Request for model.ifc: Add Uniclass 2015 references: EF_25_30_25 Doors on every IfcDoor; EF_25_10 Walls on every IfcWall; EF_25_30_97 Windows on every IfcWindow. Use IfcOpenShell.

First a look at what the model holds.

```python
import ifcopenshell

model = ifcopenshell.open("model.ifc")
print(model.schema)
print("classifications:", [c.Name for c in model.by_type("IfcClassification")])
for ifc_class in ("IfcDoor", "IfcRoof", "IfcStair", "IfcWall", "IfcWindow"):
    print(ifc_class, len(model.by_type(ifc_class)))
```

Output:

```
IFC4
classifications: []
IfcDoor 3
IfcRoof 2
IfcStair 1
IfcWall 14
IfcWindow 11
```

```python
import ifcopenshell
import ifcopenshell.api.classification

model = ifcopenshell.open("model.ifc")

system = ifcopenshell.api.classification.add_classification(model, classification="Uniclass 2015")

codes = {
    "IfcDoor": ("EF_25_30_25", "Doors"),
    "IfcWall": ("EF_25_10", "Walls"),
    "IfcWindow": ("EF_25_30_97", "Windows"),
}
for ifc_class, (code, name) in codes.items():
    products = model.by_type(ifc_class)
    ifcopenshell.api.classification.add_reference(
        model, products=products, classification=system, identification=code, name=name
    )
    print(code, len(products))

model.write("model_v2.ifc")
```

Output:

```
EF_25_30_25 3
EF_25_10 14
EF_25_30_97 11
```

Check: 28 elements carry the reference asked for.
